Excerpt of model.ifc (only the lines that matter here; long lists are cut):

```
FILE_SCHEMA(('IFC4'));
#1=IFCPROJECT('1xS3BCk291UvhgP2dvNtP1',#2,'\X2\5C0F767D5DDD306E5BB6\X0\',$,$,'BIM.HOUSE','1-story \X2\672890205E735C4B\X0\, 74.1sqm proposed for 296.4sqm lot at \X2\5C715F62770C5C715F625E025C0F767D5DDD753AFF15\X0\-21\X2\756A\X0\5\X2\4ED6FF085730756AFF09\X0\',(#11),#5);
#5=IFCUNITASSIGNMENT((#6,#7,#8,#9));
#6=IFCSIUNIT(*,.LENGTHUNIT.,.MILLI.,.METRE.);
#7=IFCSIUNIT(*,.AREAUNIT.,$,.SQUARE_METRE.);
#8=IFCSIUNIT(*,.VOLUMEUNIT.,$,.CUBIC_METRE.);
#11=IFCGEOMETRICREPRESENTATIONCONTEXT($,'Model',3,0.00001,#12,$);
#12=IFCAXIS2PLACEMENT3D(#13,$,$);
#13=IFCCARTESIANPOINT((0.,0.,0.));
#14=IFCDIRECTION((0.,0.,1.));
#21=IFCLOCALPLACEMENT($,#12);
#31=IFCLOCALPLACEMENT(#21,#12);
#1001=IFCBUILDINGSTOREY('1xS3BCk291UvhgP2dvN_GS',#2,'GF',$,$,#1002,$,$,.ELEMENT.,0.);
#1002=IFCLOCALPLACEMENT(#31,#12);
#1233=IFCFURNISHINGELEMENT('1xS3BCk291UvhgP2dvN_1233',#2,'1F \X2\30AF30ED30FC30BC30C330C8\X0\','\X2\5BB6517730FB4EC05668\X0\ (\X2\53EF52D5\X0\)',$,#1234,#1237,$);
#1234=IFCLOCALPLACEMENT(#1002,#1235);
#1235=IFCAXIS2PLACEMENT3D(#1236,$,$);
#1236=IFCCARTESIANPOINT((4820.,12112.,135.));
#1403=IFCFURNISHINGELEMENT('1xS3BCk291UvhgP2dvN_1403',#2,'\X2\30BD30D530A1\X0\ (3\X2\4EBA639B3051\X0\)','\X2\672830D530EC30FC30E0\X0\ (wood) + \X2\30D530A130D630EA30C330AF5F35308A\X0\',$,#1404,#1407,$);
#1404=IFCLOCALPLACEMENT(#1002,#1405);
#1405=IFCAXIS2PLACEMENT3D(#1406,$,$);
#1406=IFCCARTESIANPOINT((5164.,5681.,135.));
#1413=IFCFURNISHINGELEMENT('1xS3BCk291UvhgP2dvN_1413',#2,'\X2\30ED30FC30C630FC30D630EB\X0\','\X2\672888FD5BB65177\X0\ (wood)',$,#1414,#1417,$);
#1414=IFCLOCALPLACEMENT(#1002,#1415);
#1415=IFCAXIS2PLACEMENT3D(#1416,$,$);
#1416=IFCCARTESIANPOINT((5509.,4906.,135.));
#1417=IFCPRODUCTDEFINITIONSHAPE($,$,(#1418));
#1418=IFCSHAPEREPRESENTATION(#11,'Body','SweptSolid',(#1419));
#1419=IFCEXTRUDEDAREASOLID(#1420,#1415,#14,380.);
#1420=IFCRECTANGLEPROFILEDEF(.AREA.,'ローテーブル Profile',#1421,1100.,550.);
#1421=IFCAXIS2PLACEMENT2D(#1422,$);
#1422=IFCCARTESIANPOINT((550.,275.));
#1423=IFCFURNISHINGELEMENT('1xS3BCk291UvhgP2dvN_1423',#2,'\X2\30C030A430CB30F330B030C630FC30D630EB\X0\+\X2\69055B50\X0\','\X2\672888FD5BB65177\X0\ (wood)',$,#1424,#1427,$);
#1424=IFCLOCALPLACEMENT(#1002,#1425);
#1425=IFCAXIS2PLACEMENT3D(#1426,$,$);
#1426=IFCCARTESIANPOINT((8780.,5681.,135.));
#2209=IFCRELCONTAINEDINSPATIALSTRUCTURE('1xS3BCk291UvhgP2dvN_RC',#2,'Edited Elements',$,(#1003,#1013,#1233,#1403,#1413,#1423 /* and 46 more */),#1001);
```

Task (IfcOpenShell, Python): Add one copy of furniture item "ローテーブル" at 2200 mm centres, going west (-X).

```python
import numpy as np
import ifcopenshell
import ifcopenshell.api.geometry
import ifcopenshell.api.root
import ifcopenshell.util.element
import ifcopenshell.util.placement
import ifcopenshell.util.unit

model = ifcopenshell.open("model.ifc")
unit_scale = ifcopenshell.util.unit.calculate_unit_scale(model)


def reuse_history(source, copy):
    """copy_class also copies each property set's owner history, people and application; keep the originals."""
    for rel in copy.IsDefinedBy:
        if rel.is_a("IfcRelDefinesByProperties") and (history := rel.RelatingPropertyDefinition.OwnerHistory):
            rel.RelatingPropertyDefinition.OwnerHistory = source.OwnerHistory
            ifcopenshell.util.element.remove_deep2(model, history)


source = model.by_guid("1xS3BCk291UvhgP2dvN_1413")
base = ifcopenshell.util.placement.get_local_placement(source.ObjectPlacement)
step = np.array([-1.0, 0.0, 0.0]) * 2.2 / unit_scale

for i in range(1, 2):
    copy = ifcopenshell.api.root.copy_class(model, product=source)
    copy.Representation = ifcopenshell.util.element.copy_deep(
        model, source.Representation, exclude=["IfcGeometricRepresentationContext", "IfcRepresentationMap"]
    )
    reuse_history(source, copy)
    matrix = base.copy()
    matrix[:3, 3] += i * step
    print("added at", matrix[:3, 3].round(3) + 0.0)
    ifcopenshell.api.geometry.edit_object_placement(model, product=copy, matrix=matrix, is_si=False)

model.write("model_edited.ifc")
```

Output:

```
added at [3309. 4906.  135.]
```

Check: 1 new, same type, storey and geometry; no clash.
